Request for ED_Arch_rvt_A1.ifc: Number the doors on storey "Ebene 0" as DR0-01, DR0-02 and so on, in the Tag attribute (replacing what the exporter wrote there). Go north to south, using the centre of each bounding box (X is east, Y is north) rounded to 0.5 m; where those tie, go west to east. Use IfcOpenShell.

First a look at what the model holds.

```python
import ifcopenshell
import ifcopenshell.util.element
import ifcopenshell.util.placement

model = ifcopenshell.open("ED_Arch_rvt_A1.ifc")
print(model.schema)
storey = next(s for s in model.by_type("IfcBuildingStorey") if s.Name == "Ebene 0")
doors = [e for e in ifcopenshell.util.element.get_decomposition(storey) if e.is_a("IfcDoor")]
for e in sorted(doors, key=lambda e: e.id()):
    origin = ifcopenshell.util.placement.get_local_placement(e.ObjectPlacement)[:3, 3]
    print(e.id(), e.Tag, e.Name, origin.round(2) + 0.0, sep=" | ")
```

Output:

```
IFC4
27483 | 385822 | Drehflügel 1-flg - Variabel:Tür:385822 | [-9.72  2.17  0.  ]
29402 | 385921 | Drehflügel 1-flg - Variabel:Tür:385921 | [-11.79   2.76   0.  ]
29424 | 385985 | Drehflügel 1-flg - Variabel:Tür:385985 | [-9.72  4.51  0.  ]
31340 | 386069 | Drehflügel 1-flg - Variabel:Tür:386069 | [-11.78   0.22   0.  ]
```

```python
import ifcopenshell
import ifcopenshell.geom
import ifcopenshell.util.element
import ifcopenshell.util.shape

model = ifcopenshell.open("ED_Arch_rvt_A1.ifc")
settings = ifcopenshell.geom.settings()
settings.set("use-world-coords", True)


def centre(element):
    shape = ifcopenshell.geom.create_shape(settings, element)
    return ifcopenshell.util.shape.get_bbox_centroid(shape.geometry)


storey = next(s for s in model.by_type("IfcBuildingStorey") if s.Name == "Ebene 0")
doors = [e for e in ifcopenshell.util.element.get_decomposition(storey) if e.is_a("IfcDoor")]

# Insertion points can sit at a corner or the storey origin, so sort by the geometry (in metres).
centres = {e: centre(e) for e in doors}
doors.sort(key=lambda e: (-round(centres[e][1] / 0.5), centres[e][0]))

for i, e in enumerate(doors, start=1):
    number = f"DR0-{i:02d}"
    e.Tag = number
    print(e.id(), number)

model.write("ED_Arch_rvt_A1-out.ifc")
```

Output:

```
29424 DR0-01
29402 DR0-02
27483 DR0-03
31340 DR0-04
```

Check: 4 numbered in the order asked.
